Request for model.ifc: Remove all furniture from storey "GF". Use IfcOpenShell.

First a look at what the model holds.

```python
import ifcopenshell
import ifcopenshell.util.element

model = ifcopenshell.open("model.ifc")
print(model.schema)
storey = next(s for s in model.by_type("IfcBuildingStorey") if s.Name == "GF")
furniture = [e for e in ifcopenshell.util.element.get_decomposition(storey) if e.is_a("IfcFurnishingElement")]
seen = {}
for e in furniture:
    element_type = ifcopenshell.util.element.get_type(e)
    name = element_type.Name if element_type not in (None, e) else None
    seen[name] = seen.get(name, 0) + 1
for name, count in sorted(seen.items(), key=str):
    print(count, "x", name)
```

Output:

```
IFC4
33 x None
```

```python
import ifcopenshell
import ifcopenshell.api.root
import ifcopenshell.util.element

model = ifcopenshell.open("model.ifc")

storey = next(s for s in model.by_type("IfcBuildingStorey") if s.Name == "GF")
furniture = [e for e in ifcopenshell.util.element.get_decomposition(storey) if e.is_a("IfcFurnishingElement")]

for e in furniture:
    ifcopenshell.api.root.remove_product(model, product=e)
print(len(furniture), "removed")

model.write("model_updated.ifc")
```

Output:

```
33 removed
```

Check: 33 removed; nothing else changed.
